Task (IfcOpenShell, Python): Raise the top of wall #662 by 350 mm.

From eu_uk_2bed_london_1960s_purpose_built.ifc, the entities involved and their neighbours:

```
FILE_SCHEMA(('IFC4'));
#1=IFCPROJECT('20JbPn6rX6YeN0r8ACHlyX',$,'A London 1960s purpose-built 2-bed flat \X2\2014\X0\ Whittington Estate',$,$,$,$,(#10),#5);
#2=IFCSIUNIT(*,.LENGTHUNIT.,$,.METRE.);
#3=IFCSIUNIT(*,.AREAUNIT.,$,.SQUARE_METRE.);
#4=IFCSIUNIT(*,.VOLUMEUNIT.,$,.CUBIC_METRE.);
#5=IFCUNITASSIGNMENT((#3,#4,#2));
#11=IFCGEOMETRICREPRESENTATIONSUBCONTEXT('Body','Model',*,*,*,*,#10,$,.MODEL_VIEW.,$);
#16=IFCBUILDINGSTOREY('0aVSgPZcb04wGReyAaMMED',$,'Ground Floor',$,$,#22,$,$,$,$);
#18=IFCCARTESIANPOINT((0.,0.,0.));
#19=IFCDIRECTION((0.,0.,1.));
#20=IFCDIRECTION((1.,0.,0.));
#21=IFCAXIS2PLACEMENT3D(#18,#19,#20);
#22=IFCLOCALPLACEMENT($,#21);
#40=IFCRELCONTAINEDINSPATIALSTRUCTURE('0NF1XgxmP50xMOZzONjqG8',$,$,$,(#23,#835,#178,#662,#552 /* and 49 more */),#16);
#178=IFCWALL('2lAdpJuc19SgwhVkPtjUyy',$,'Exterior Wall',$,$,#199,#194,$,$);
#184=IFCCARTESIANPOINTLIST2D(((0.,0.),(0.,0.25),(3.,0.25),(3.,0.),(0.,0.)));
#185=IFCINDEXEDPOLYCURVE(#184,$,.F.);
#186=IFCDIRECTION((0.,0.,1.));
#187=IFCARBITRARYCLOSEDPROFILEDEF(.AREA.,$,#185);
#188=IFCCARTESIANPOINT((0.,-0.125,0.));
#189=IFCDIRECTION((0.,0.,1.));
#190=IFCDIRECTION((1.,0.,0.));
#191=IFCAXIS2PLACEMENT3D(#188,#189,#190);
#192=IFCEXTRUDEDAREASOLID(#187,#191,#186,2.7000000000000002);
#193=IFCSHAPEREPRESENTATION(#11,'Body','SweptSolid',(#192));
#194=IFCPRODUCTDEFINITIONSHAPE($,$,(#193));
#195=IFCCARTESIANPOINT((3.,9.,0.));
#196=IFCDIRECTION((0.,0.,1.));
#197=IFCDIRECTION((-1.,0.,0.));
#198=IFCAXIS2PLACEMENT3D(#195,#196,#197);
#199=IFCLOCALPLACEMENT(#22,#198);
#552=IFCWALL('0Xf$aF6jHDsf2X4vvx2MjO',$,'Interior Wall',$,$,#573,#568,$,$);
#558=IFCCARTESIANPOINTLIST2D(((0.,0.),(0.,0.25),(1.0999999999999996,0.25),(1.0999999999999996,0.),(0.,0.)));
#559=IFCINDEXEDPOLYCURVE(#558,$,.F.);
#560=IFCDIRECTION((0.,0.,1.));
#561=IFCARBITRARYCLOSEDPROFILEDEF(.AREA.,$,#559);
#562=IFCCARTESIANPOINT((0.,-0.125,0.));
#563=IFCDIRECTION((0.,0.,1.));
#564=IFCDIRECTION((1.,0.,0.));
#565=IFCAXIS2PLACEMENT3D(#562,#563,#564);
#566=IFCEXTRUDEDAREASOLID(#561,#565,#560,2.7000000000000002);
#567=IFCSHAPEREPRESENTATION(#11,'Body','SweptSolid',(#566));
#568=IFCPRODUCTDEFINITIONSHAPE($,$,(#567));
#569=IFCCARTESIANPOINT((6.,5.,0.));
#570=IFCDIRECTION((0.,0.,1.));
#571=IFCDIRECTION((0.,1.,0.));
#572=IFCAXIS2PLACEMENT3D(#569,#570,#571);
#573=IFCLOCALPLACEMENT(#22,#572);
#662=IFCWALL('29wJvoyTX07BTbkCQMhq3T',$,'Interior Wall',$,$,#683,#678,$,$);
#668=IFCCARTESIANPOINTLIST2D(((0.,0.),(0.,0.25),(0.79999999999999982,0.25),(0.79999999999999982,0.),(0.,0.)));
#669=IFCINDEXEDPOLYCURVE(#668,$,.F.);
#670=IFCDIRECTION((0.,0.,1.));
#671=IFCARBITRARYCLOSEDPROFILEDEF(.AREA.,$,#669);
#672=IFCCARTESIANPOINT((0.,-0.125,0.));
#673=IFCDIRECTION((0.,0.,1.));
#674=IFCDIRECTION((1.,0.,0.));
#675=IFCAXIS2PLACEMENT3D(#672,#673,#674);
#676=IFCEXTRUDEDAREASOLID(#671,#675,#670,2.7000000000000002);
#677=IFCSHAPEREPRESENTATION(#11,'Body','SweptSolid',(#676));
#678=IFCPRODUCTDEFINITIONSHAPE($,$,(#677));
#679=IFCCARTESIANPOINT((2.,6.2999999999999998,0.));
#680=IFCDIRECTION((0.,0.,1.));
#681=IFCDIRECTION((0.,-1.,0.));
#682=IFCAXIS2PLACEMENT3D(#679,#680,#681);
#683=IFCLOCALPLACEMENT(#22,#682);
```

```python
import ifcopenshell
import ifcopenshell.geom
import ifcopenshell.util.representation
import ifcopenshell.util.shape
import ifcopenshell.util.unit

model = ifcopenshell.open("eu_uk_2bed_london_1960s_purpose_built.ifc")
unit_scale = ifcopenshell.util.unit.calculate_unit_scale(model)
settings = ifcopenshell.geom.settings()


def volume(element):
    """Net volume in cubic metres, openings subtracted."""
    shape = ifcopenshell.geom.create_shape(settings, element)
    return ifcopenshell.util.shape.get_volume(shape.geometry)


wall = model.by_guid("29wJvoyTX07BTbkCQMhq3T")
before = volume(wall)

body = ifcopenshell.util.representation.get_representation(wall, "Model", "Body")
solid = body.Items[0]
old_height = solid.Depth
solid.Depth += 0.35 / unit_scale
after = volume(wall)

print(f"height {old_height:g} -> {solid.Depth:g}, volume {before:.3f} -> {after:.3f} m3")

model.write("eu_uk_2bed_london_1960s_purpose_built_updated.ifc")
```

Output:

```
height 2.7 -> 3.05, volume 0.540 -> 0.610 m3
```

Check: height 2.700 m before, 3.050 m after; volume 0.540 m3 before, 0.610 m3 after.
